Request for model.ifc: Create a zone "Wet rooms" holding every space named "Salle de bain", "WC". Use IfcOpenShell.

First a look at what the model holds.

```python
import ifcopenshell

model = ifcopenshell.open("model.ifc")
print(model.schema)
seen = {}
for space in model.by_type("IfcSpace"):
    seen[space.LongName] = seen.get(space.LongName, 0) + 1
for name, count in sorted(seen.items(), key=str):
    print(count, "x", name)
print("zones:", [z.Name for z in model.by_type("IfcZone")][:20])
```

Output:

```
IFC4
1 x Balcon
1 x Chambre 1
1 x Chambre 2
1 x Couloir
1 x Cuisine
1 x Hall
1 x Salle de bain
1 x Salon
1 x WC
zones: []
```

```python
import ifcopenshell
import ifcopenshell.api.group
import ifcopenshell.api.root

model = ifcopenshell.open("model.ifc")

names = {"Salle de bain", "WC"}
spaces = [s for s in model.by_type("IfcSpace") if s.LongName in names]

zone = ifcopenshell.api.root.create_entity(model, ifc_class="IfcZone", name="Wet rooms")
ifcopenshell.api.group.assign_group(model, products=spaces, group=zone)
print(len(spaces), "spaces in", zone.Name)

model.write("model_updated.ifc")
```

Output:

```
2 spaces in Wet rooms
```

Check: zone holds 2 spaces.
